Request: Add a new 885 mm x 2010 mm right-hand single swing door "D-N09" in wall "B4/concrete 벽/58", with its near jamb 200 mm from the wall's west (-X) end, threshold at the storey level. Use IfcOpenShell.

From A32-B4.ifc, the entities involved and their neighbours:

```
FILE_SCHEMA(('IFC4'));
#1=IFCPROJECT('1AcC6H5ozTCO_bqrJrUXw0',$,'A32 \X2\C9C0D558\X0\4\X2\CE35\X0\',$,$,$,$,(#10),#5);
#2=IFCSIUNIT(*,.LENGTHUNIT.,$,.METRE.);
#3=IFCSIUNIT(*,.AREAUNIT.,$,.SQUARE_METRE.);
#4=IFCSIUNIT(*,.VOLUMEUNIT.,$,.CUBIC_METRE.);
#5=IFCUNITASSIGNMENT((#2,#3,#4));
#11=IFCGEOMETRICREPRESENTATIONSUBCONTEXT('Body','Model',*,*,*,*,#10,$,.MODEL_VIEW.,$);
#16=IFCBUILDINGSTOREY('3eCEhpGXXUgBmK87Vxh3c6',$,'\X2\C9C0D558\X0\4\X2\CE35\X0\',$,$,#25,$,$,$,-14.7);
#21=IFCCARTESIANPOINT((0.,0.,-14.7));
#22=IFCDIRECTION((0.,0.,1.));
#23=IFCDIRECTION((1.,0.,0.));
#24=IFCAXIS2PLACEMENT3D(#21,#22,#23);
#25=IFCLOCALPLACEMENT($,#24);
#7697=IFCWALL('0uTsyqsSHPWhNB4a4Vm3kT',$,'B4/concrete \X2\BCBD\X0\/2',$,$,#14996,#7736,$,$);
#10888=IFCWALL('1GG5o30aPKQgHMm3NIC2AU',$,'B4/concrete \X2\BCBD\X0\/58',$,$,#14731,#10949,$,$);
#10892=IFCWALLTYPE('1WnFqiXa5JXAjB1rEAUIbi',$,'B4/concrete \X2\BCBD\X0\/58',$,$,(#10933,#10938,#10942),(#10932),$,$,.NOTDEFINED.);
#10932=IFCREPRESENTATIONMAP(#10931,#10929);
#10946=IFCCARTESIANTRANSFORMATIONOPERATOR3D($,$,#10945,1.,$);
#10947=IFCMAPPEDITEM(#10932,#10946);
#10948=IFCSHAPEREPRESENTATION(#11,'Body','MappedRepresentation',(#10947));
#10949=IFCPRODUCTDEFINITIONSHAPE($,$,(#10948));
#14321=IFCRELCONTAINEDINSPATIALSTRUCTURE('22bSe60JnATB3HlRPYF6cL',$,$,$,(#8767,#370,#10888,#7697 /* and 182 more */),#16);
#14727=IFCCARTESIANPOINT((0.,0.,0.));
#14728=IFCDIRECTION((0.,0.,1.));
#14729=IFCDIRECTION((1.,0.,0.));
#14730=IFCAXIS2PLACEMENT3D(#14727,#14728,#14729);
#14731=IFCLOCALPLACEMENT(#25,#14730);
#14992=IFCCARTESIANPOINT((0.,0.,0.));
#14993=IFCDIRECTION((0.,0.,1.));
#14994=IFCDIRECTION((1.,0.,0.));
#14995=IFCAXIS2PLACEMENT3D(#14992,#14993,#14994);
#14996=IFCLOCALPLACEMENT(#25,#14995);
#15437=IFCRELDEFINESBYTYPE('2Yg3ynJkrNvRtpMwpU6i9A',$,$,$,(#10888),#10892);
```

```python
import numpy as np
import ifcopenshell
import ifcopenshell.api.feature
import ifcopenshell.api.geometry
import ifcopenshell.api.root
import ifcopenshell.api.spatial
import ifcopenshell.geom
import ifcopenshell.util.element
import ifcopenshell.util.placement
import ifcopenshell.util.representation
import ifcopenshell.util.shape
import ifcopenshell.util.unit

model = ifcopenshell.open("A32-B4.ifc")
unit_scale = ifcopenshell.util.unit.calculate_unit_scale(model)
settings = ifcopenshell.geom.settings()


def volume(element):
    """Net volume in cubic metres, openings subtracted."""
    shape = ifcopenshell.geom.create_shape(settings, element)
    return ifcopenshell.util.shape.get_volume(shape.geometry)


wall = model.by_guid("1GG5o30aPKQgHMm3NIC2AU")
storey = ifcopenshell.util.element.get_container(wall, ifc_class="IfcBuildingStorey")
context = ifcopenshell.util.representation.get_context(model, "Model", "Body", "MODEL_VIEW")
before = volume(wall)

width, height, from_end, sill = 0.885, 2.01, 0.2, 0.0  # metres

# The wall runs along its own X axis, and the end named is its -X end.
wall_shape = ifcopenshell.geom.create_shape(settings, wall)
x, y, z = ifcopenshell.util.shape.get_vertices(wall_shape.geometry).T
start = x.min() + from_end
face, thickness = float(y.min()), float(y.max() - y.min())
wall_matrix = ifcopenshell.util.placement.get_local_placement(wall.ObjectPlacement)
level = ifcopenshell.util.placement.get_local_placement(storey.ObjectPlacement)[2, 3]


def in_wall(x, y):
    """Placement at x, y metres in the wall's axes, at sill height."""
    matrix = wall_matrix.copy()
    matrix[:, 3] = wall_matrix @ np.array([x / unit_scale, y / unit_scale, 0.0, 1.0])
    matrix[2, 3] = level + sill / unit_scale
    return matrix


# Opening: a box that overshoots both wall faces by 50 mm.
opening = ifcopenshell.api.root.create_entity(model, ifc_class="IfcOpeningElement", predefined_type="OPENING")
box = ifcopenshell.api.geometry.add_wall_representation(
    model, context=context, length=width, height=height, thickness=thickness + 0.1
)
ifcopenshell.api.geometry.assign_representation(model, product=opening, representation=box)
ifcopenshell.api.geometry.edit_object_placement(model, product=opening, matrix=in_wall(start, face - 0.05), is_si=False)
ifcopenshell.api.feature.add_feature(model, feature=opening, element=wall)

door = ifcopenshell.api.root.create_entity(model, ifc_class="IfcDoor", name="D-N09", predefined_type="DOOR")
door.OverallWidth, door.OverallHeight = width / unit_scale, height / unit_scale
door.OperationType = "SINGLE_SWING_RIGHT"
body = ifcopenshell.api.geometry.add_door_representation(
    model,
    context=context,
    overall_width=door.OverallWidth,
    overall_height=door.OverallHeight,
    operation_type="SINGLE_SWING_RIGHT",
    lining_properties={"LiningDepth": thickness / unit_scale, "ThresholdDepth": thickness / unit_scale},
)
ifcopenshell.api.geometry.assign_representation(model, product=door, representation=body)
ifcopenshell.api.spatial.assign_container(model, products=[door], relating_structure=storey)
ifcopenshell.api.feature.add_filling(model, opening=opening, element=door)

# The lining spans the wall, so the door starts at the wall face.
ifcopenshell.api.geometry.edit_object_placement(model, product=door, matrix=in_wall(start, face), is_si=False)

after = volume(wall)

print(f"wall volume {before:.3f} -> {after:.3f} m3")

model.write("A32-B4_rev.ifc")
```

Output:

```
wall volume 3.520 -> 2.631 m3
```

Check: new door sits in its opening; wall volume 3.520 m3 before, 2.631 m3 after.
